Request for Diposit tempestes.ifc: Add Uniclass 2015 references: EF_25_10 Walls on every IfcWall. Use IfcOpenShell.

First a look at what the model holds.

```python
import ifcopenshell

model = ifcopenshell.open("Diposit tempestes.ifc")
print(model.schema)
print("classifications:", [c.Name for c in model.by_type("IfcClassification")])
for ifc_class in ("IfcDoor", "IfcRoof", "IfcStair", "IfcWall", "IfcWindow"):
    print(ifc_class, len(model.by_type(ifc_class)))
```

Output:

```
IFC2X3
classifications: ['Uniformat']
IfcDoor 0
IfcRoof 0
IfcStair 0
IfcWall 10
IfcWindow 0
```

```python
import ifcopenshell
import ifcopenshell.api.classification

model = ifcopenshell.open("Diposit tempestes.ifc")

# IFC2X3 requires Source and Edition and has no link from the project to the system.
system = model.create_entity("IfcClassification", Source="NBS", Edition="2015", Name="Uniclass 2015")

codes = {
    "IfcWall": ("EF_25_10", "Walls"),
}
for ifc_class, (code, name) in codes.items():
    products = model.by_type(ifc_class)
    ifcopenshell.api.classification.add_reference(
        model, products=products, classification=system, identification=code, name=name
    )
    print(code, len(products))

model.write("Diposit tempestes_updated.ifc")
```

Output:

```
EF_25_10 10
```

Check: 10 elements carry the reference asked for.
